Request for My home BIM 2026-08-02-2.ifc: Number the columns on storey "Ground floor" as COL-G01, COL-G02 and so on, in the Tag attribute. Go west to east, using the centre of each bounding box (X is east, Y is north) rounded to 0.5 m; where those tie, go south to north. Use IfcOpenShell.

First a look at what the model holds.

```python
import ifcopenshell
import ifcopenshell.util.element
import ifcopenshell.util.placement

model = ifcopenshell.open("My home BIM 2026-08-02-2.ifc")
print(model.schema)
storey = next(s for s in model.by_type("IfcBuildingStorey") if s.Name == "Ground floor")
columns = [e for e in ifcopenshell.util.element.get_decomposition(storey) if e.is_a("IfcColumn")]
for e in sorted(columns, key=lambda e: e.id()):
    origin = ifcopenshell.util.placement.get_local_placement(e.ObjectPlacement)[:3, 3]
    print(e.id(), e.Tag, e.Name, origin.round(2) + 0.0, sep=" | ")
```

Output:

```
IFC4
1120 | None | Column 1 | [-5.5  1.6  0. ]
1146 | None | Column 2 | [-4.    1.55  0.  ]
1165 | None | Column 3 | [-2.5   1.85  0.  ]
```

```python
import ifcopenshell
import ifcopenshell.geom
import ifcopenshell.util.element
import ifcopenshell.util.shape

model = ifcopenshell.open("My home BIM 2026-08-02-2.ifc")
settings = ifcopenshell.geom.settings()
settings.set("use-world-coords", True)


def centre(element):
    shape = ifcopenshell.geom.create_shape(settings, element)
    return ifcopenshell.util.shape.get_bbox_centroid(shape.geometry)


storey = next(s for s in model.by_type("IfcBuildingStorey") if s.Name == "Ground floor")
columns = [e for e in ifcopenshell.util.element.get_decomposition(storey) if e.is_a("IfcColumn")]

# Insertion points can sit at a corner or the storey origin, so sort by the geometry (in metres).
centres = {e: centre(e) for e in columns}
columns.sort(key=lambda e: (round(centres[e][0] / 0.5), centres[e][1]))

for i, e in enumerate(columns, start=1):
    number = f"COL-G{i:02d}"
    e.Tag = number
    print(e.id(), number)

model.write("My home BIM 2026-08-02-2_edited.ifc")
```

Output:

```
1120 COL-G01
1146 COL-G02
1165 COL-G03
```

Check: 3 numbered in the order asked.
